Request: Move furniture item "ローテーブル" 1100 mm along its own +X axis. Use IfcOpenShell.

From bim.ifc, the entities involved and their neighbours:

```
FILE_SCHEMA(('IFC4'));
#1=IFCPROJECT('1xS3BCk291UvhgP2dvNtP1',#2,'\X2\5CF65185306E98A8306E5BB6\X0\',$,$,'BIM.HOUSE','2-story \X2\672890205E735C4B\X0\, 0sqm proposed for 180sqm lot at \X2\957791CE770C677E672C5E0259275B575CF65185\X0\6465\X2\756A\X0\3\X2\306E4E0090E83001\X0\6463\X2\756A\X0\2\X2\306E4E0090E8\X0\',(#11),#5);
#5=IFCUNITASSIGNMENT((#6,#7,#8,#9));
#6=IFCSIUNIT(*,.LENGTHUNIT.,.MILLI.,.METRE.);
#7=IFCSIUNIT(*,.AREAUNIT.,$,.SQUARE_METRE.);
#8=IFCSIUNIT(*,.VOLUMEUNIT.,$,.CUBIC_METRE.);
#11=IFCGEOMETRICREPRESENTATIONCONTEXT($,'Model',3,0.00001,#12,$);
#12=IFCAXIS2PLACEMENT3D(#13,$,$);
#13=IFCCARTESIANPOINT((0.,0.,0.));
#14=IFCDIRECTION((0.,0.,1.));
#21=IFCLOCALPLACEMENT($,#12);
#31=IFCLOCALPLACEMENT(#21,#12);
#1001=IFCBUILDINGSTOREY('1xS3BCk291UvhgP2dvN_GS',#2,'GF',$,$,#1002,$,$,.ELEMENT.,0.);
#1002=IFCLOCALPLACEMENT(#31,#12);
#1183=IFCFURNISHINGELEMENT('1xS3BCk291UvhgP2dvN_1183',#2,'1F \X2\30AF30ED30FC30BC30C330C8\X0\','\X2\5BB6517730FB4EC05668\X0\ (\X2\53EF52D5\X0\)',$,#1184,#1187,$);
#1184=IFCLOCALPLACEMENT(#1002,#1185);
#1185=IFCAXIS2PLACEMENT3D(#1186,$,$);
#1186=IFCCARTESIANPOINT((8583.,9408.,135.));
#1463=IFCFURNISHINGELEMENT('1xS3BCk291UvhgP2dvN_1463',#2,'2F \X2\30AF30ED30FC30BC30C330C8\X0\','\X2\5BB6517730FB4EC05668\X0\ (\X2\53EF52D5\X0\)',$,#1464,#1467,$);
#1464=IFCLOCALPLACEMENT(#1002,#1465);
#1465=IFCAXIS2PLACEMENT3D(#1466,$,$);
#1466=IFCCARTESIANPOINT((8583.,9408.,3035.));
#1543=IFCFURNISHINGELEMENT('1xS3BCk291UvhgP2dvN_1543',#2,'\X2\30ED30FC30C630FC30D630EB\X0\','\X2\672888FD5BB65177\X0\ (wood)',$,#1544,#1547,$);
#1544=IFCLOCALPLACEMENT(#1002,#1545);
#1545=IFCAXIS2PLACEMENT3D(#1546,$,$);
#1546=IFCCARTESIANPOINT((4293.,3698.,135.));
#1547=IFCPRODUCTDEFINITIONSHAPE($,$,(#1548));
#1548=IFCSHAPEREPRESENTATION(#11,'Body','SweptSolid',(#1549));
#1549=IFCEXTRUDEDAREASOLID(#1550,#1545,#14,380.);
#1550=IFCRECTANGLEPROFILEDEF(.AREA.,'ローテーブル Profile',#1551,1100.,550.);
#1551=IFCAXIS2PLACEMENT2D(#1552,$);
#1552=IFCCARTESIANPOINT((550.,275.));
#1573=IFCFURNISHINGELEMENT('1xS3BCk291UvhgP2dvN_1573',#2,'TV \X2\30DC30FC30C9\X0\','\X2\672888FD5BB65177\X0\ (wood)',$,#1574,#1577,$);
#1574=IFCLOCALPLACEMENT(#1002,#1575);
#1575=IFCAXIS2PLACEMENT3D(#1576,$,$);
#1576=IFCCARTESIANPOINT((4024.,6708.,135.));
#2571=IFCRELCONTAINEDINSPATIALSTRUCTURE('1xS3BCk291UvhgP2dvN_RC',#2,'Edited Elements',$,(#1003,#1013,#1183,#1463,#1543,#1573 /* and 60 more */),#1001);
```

```python
import ifcopenshell
import ifcopenshell.api.geometry
import ifcopenshell.util.placement

model = ifcopenshell.open("bim.ifc")

item = model.by_guid("1xS3BCk291UvhgP2dvN_1543")
matrix = ifcopenshell.util.placement.get_local_placement(item.ObjectPlacement)
matrix[:3, 3] += matrix[:3, 0] * 1100.0
ifcopenshell.api.geometry.edit_object_placement(model, product=item, matrix=matrix, is_si=False)

print(ifcopenshell.util.placement.get_local_placement(item.ObjectPlacement).round(3) + 0.0)

model.write("bim_v2.ifc")
```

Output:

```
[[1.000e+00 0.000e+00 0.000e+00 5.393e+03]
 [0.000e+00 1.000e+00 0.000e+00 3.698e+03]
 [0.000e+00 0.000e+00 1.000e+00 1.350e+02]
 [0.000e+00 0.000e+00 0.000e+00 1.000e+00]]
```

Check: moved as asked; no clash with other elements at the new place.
